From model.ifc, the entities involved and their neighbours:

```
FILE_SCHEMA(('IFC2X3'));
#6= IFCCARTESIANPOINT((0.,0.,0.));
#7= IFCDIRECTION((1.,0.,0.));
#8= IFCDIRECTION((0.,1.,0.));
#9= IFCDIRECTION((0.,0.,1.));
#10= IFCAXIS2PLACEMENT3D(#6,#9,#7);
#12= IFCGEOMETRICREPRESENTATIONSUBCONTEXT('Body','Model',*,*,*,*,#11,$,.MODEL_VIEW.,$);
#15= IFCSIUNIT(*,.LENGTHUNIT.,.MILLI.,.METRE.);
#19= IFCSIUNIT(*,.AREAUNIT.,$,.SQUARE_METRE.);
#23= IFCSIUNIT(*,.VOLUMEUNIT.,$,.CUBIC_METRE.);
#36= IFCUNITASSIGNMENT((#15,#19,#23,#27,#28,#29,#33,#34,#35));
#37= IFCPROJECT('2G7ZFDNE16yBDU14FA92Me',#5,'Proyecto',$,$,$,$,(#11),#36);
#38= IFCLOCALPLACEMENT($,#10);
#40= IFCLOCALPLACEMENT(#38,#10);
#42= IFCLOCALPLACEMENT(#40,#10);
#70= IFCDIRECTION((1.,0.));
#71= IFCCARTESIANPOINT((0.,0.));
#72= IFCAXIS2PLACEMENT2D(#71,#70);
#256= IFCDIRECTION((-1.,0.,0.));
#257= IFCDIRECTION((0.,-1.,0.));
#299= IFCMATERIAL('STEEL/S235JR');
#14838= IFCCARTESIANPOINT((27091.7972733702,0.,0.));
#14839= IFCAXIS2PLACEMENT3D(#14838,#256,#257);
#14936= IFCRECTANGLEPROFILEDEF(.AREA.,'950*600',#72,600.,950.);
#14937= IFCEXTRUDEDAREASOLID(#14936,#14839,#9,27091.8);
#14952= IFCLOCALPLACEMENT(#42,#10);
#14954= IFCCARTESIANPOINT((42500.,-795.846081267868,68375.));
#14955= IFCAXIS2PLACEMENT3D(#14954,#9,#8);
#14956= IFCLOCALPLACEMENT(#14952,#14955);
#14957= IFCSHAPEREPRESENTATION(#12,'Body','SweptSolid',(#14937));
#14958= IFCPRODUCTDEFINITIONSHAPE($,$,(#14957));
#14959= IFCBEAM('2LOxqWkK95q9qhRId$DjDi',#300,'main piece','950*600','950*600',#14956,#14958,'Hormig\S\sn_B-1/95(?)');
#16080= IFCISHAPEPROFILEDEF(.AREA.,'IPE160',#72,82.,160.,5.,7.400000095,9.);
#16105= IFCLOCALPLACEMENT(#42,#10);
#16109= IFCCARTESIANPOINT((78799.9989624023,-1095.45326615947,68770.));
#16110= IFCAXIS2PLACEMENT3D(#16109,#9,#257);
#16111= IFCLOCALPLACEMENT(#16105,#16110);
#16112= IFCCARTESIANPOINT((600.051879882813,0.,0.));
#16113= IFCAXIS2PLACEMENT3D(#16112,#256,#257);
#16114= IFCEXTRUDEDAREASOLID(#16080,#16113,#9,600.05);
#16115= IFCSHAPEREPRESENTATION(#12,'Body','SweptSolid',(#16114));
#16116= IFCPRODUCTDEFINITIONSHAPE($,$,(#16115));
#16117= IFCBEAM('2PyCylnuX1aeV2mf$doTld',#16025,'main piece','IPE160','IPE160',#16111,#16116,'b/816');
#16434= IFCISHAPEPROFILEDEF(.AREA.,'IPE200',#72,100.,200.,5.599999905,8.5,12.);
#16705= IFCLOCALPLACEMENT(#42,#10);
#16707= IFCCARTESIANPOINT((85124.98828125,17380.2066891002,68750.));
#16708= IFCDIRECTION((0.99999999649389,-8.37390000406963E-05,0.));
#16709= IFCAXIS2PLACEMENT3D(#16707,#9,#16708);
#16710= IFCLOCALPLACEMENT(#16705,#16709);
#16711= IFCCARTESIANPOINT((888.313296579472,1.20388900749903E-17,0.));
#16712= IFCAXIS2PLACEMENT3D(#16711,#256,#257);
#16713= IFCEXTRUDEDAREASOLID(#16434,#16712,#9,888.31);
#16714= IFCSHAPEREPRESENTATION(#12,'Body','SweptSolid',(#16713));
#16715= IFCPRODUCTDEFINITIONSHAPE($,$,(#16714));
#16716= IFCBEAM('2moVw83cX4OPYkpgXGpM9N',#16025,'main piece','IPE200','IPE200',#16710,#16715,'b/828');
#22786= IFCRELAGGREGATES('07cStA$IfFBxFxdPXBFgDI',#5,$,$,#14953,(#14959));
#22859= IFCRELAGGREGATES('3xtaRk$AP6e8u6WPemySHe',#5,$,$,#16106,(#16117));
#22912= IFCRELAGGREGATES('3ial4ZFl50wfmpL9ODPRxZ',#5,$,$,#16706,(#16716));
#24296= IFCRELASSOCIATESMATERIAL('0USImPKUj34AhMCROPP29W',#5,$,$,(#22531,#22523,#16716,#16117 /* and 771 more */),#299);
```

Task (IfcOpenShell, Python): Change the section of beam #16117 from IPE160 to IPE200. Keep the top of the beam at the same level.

```python
import ifcopenshell
import ifcopenshell.util.element
import ifcopenshell.util.representation

model = ifcopenshell.open("model.ifc")

member = model.by_guid("2PyCylnuX1aeV2mf$doTld")
source = next(p for p in model.by_type("IfcIShapeProfileDef") if p.ProfileName == "IPE200")

body = ifcopenshell.util.representation.get_representation(member, "Model", "Body")
solid = body.Items[0]
old_profile = solid.SweptArea

# Copy the section's sizes but keep this member's own profile position.
profile = ifcopenshell.util.element.copy(model, source)
# Profiles are centred, so shift by half the change in depth to hold the top.
shift = (old_profile.OverallDepth - profile.OverallDepth) / 2
x, y = old_profile.Position.Location.Coordinates
up = (0.0, 1.0)  # upwards, in the solid's own plane
location = model.createIfcCartesianPoint((x + up[0] * shift, y + up[1] * shift))
profile.Position = model.createIfcAxis2Placement2D(location, old_profile.Position.RefDirection)
solid.SweptArea = profile
if not model.get_total_inverses(old_profile):
    ifcopenshell.util.element.remove_deep2(model, old_profile)
member.Description = member.Description.replace("IPE160", "IPE200")
member.ObjectType = member.ObjectType.replace("IPE160", "IPE200")

print(solid.SweptArea)

model.write("model_updated.ifc")
```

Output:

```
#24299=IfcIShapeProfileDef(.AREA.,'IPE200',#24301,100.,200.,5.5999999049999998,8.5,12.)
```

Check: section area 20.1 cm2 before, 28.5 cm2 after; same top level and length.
